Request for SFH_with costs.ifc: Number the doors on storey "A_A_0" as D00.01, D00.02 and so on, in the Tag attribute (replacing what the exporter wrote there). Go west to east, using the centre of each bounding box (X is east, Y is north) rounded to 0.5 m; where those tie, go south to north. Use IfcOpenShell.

First a look at what the model holds.

```python
import ifcopenshell
import ifcopenshell.util.element
import ifcopenshell.util.placement

model = ifcopenshell.open("SFH_with costs.ifc")
print(model.schema)
storey = next(s for s in model.by_type("IfcBuildingStorey") if s.Name == "A_A_0")
doors = [e for e in ifcopenshell.util.element.get_decomposition(storey) if e.is_a("IfcDoor")]
for e in sorted(doors, key=lambda e: e.id()):
    origin = ifcopenshell.util.placement.get_local_placement(e.ObjectPlacement)[:3, 3]
    print(e.id(), e.Tag, e.Name, origin.round(2) + 0.0, sep=" | ")
```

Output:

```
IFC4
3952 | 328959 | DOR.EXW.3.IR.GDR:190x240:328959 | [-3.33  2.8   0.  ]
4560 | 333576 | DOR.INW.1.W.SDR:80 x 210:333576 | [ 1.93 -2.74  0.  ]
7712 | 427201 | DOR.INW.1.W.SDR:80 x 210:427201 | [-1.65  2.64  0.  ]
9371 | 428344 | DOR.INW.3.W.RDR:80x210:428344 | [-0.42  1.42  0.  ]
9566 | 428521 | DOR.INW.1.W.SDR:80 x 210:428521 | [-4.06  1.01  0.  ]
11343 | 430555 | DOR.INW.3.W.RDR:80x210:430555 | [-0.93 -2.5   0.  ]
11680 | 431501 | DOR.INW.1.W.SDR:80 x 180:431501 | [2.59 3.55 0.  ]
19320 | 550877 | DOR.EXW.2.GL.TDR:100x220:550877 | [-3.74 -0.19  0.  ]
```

```python
import ifcopenshell
import ifcopenshell.geom
import ifcopenshell.util.element
import ifcopenshell.util.shape

model = ifcopenshell.open("SFH_with costs.ifc")
settings = ifcopenshell.geom.settings()
settings.set("use-world-coords", True)


def centre(element):
    shape = ifcopenshell.geom.create_shape(settings, element)
    return ifcopenshell.util.shape.get_bbox_centroid(shape.geometry)


storey = next(s for s in model.by_type("IfcBuildingStorey") if s.Name == "A_A_0")
doors = [e for e in ifcopenshell.util.element.get_decomposition(storey) if e.is_a("IfcDoor")]

# Insertion points can sit at a corner or the storey origin, so sort by the geometry (in metres).
centres = {e: centre(e) for e in doors}
doors.sort(key=lambda e: (round(centres[e][0] / 0.5), centres[e][1]))

for i, e in enumerate(doors, start=1):
    number = f"D00.{i:02d}"
    e.Tag = number
    print(e.id(), number)

model.write("SFH_with costs_updated.ifc")
```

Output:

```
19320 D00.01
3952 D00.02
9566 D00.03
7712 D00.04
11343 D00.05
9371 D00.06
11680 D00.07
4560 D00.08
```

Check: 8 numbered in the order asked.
